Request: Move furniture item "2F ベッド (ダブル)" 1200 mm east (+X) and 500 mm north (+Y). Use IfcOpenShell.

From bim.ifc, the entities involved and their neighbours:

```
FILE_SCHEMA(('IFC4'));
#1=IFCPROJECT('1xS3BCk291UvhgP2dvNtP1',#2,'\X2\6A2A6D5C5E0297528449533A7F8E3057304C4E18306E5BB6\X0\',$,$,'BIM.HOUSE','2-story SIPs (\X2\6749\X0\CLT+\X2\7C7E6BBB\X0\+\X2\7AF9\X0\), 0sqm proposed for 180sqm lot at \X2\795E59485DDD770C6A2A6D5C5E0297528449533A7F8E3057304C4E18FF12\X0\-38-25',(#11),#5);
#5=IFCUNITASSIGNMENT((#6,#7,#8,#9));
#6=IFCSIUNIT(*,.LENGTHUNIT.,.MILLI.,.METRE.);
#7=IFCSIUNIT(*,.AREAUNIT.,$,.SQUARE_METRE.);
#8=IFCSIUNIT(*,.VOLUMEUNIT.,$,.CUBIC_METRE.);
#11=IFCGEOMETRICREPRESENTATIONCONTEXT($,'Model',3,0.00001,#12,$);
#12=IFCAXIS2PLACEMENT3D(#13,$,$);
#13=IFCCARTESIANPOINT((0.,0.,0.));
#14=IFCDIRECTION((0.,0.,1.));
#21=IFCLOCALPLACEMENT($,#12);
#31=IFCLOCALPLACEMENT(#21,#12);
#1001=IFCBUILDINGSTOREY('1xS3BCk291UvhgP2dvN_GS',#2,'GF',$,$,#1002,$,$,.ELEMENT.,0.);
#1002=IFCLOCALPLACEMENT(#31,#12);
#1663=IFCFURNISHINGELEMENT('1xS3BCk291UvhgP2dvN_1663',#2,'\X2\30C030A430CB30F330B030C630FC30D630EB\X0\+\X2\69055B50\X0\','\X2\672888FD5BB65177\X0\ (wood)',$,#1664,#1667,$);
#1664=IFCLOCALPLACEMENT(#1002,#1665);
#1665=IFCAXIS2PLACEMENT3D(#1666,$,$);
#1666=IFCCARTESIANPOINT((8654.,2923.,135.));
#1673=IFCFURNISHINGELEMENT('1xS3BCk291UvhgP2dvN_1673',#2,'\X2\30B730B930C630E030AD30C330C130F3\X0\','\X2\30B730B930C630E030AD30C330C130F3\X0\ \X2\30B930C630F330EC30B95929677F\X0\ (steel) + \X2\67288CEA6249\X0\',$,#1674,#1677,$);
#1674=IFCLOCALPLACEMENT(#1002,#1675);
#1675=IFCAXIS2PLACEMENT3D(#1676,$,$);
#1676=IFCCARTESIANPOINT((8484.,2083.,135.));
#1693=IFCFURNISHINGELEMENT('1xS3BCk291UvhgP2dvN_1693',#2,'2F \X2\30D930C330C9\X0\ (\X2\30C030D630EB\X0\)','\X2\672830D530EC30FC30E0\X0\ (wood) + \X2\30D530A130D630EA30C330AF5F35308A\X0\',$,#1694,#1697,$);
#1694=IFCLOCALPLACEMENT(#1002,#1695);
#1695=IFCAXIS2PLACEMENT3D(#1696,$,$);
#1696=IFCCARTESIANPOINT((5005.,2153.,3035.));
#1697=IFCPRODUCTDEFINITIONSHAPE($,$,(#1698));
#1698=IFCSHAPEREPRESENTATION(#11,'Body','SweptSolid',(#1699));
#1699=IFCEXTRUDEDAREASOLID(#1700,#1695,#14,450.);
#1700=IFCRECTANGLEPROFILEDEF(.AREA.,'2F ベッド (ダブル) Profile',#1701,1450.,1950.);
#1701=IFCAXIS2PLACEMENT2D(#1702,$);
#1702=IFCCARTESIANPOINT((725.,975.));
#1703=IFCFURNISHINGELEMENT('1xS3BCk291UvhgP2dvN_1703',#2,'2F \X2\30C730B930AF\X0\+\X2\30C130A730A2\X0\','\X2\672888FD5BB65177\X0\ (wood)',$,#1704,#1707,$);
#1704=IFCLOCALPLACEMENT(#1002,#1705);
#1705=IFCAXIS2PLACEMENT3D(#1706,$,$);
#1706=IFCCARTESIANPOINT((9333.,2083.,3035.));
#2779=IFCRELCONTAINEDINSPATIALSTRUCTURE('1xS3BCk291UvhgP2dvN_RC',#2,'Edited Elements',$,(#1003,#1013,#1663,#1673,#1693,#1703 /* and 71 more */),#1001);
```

```python
import ifcopenshell
import ifcopenshell.api.geometry
import ifcopenshell.util.placement

model = ifcopenshell.open("bim.ifc")

item = model.by_id(1693)
matrix = ifcopenshell.util.placement.get_local_placement(item.ObjectPlacement)
matrix[0, 3] += 1200.0
matrix[1, 3] += 500.0
ifcopenshell.api.geometry.edit_object_placement(model, product=item, matrix=matrix, is_si=False)

print(ifcopenshell.util.placement.get_local_placement(item.ObjectPlacement).round(3) + 0.0)

model.write("bim_updated.ifc")
```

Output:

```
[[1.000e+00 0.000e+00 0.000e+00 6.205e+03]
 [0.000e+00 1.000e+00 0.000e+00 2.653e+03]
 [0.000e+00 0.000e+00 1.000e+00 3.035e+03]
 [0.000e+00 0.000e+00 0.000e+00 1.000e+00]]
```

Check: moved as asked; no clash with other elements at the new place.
